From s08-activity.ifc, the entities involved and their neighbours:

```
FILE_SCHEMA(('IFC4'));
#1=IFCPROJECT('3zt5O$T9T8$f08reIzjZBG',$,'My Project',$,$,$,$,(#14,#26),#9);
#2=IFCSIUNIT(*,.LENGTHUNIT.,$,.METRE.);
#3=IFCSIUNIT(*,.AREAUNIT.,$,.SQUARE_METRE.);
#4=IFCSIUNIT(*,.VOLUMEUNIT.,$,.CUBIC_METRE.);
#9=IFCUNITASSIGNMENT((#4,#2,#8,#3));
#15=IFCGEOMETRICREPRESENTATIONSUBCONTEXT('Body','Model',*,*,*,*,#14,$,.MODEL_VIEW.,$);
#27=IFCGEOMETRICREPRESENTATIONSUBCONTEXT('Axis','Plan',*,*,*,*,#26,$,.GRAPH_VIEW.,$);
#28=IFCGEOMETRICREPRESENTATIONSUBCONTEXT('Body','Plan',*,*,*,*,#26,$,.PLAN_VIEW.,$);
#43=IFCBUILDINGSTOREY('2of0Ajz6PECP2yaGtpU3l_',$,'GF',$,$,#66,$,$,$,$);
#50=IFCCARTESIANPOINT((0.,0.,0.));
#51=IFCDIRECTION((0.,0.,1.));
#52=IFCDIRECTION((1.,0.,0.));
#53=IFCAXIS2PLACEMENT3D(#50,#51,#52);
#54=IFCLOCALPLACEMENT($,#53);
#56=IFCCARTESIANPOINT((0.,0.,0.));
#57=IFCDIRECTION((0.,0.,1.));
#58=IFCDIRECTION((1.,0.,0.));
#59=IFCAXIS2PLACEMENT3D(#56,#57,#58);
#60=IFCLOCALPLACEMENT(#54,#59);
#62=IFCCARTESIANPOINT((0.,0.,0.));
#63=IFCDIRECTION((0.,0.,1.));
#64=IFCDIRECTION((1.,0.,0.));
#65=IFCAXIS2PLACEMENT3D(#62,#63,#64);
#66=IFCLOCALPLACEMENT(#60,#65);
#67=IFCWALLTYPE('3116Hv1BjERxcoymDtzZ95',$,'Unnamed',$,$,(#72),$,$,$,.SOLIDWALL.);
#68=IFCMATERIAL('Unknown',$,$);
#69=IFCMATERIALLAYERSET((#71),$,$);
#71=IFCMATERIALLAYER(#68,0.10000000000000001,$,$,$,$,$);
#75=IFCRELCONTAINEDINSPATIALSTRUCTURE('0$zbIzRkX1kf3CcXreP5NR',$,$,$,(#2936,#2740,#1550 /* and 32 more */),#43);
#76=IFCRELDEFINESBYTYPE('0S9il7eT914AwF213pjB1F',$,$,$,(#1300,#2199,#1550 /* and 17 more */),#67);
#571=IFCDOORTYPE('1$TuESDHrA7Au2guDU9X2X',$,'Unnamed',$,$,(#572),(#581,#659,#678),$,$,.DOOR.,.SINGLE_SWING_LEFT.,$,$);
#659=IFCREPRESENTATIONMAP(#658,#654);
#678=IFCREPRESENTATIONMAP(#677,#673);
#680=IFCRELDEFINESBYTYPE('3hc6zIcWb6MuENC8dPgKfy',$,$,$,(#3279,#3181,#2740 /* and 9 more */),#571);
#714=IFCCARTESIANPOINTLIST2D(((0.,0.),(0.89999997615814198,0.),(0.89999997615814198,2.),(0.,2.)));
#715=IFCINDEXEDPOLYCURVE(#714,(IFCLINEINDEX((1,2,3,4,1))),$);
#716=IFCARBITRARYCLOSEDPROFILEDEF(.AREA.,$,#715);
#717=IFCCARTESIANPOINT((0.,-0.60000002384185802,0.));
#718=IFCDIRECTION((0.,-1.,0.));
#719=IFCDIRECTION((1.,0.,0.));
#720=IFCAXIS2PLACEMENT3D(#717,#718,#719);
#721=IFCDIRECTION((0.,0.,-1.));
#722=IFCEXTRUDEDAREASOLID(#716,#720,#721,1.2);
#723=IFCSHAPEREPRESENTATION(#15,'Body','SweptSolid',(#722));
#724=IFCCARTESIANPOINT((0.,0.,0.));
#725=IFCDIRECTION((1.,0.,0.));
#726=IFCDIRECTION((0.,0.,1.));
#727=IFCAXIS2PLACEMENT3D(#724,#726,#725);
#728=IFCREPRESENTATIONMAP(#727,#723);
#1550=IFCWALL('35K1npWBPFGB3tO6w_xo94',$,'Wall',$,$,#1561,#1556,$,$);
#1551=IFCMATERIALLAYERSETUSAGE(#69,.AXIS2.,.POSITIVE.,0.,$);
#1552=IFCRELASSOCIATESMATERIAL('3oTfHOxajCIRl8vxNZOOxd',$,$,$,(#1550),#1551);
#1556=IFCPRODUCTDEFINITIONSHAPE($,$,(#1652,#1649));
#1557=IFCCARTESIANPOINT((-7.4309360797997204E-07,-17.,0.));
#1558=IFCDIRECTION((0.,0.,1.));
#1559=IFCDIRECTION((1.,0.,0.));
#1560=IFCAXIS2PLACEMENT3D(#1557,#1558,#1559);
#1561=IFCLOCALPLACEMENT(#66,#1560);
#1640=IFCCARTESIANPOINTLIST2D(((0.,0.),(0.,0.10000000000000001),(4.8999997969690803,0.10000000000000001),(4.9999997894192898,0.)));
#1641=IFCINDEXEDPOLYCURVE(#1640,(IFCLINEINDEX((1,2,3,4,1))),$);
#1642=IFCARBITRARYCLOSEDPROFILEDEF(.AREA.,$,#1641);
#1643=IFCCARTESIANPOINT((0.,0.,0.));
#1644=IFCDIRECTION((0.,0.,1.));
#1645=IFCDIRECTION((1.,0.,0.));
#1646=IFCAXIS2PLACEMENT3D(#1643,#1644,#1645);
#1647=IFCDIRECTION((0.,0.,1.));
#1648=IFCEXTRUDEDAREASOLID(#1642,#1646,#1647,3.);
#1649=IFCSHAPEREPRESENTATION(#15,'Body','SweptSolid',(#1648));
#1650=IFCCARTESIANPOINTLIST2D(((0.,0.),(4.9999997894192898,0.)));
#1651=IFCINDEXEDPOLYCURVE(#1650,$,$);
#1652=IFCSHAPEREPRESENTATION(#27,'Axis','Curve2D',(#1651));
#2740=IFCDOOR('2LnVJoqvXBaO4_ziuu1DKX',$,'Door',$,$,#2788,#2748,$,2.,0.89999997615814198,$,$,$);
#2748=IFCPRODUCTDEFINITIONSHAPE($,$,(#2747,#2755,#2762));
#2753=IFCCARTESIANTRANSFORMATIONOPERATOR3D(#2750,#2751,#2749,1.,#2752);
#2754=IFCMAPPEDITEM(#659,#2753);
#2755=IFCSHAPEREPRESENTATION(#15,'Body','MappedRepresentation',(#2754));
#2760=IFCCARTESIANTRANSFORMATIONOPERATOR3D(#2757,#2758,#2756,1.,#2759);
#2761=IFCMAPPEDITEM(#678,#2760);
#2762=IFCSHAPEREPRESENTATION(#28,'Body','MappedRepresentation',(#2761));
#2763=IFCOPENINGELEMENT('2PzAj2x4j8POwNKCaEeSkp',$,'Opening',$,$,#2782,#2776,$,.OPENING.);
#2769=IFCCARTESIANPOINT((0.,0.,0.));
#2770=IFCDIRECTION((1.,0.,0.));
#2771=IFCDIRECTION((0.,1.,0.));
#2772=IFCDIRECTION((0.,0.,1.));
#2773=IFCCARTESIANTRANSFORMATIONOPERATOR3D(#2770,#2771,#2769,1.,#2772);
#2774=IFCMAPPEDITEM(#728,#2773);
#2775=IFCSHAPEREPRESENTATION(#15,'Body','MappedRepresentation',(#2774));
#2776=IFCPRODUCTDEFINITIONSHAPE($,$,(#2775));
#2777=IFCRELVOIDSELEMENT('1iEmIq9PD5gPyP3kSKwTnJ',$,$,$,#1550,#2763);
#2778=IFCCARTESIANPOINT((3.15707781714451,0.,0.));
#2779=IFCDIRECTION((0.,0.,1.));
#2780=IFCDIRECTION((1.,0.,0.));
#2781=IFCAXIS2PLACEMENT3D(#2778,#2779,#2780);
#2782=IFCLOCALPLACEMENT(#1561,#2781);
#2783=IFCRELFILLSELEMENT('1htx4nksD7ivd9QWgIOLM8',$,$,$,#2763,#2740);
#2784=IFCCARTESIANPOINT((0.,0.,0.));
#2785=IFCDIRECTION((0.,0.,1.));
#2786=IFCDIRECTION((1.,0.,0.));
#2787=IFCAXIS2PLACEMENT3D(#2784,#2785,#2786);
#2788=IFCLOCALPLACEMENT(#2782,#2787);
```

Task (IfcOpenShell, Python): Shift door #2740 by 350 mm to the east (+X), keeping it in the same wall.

```python
import ifcopenshell
import ifcopenshell.api.geometry
import ifcopenshell.util.placement
import ifcopenshell.util.unit

model = ifcopenshell.open("s08-activity.ifc")
unit_scale = ifcopenshell.util.unit.calculate_unit_scale(model)

door = model.by_guid("2LnVJoqvXBaO4_ziuu1DKX")
opening = door.FillsVoids[0].RelatingOpeningElement
wall = opening.VoidsElements[0].RelatingBuildingElement

wall_matrix = ifcopenshell.util.placement.get_local_placement(wall.ObjectPlacement)
shift = wall_matrix[:3, 0] * 0.35 / unit_scale
before = ifcopenshell.util.placement.get_local_placement(door.ObjectPlacement)[:3, 3].copy()

# The door is placed relative to its opening, so it follows when the opening moves.
matrix = ifcopenshell.util.placement.get_local_placement(opening.ObjectPlacement)
matrix[:3, 3] += shift
ifcopenshell.api.geometry.edit_object_placement(
    model, product=opening, matrix=matrix, is_si=False, should_transform_children=True
)

after = ifcopenshell.util.placement.get_local_placement(door.ObjectPlacement)[:3, 3]
print("door moved by", (after - before).round(3) + 0.0)

model.write("s08-activity_rev.ifc")
```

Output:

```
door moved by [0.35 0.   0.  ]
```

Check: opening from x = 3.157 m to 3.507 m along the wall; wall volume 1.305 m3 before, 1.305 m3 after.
